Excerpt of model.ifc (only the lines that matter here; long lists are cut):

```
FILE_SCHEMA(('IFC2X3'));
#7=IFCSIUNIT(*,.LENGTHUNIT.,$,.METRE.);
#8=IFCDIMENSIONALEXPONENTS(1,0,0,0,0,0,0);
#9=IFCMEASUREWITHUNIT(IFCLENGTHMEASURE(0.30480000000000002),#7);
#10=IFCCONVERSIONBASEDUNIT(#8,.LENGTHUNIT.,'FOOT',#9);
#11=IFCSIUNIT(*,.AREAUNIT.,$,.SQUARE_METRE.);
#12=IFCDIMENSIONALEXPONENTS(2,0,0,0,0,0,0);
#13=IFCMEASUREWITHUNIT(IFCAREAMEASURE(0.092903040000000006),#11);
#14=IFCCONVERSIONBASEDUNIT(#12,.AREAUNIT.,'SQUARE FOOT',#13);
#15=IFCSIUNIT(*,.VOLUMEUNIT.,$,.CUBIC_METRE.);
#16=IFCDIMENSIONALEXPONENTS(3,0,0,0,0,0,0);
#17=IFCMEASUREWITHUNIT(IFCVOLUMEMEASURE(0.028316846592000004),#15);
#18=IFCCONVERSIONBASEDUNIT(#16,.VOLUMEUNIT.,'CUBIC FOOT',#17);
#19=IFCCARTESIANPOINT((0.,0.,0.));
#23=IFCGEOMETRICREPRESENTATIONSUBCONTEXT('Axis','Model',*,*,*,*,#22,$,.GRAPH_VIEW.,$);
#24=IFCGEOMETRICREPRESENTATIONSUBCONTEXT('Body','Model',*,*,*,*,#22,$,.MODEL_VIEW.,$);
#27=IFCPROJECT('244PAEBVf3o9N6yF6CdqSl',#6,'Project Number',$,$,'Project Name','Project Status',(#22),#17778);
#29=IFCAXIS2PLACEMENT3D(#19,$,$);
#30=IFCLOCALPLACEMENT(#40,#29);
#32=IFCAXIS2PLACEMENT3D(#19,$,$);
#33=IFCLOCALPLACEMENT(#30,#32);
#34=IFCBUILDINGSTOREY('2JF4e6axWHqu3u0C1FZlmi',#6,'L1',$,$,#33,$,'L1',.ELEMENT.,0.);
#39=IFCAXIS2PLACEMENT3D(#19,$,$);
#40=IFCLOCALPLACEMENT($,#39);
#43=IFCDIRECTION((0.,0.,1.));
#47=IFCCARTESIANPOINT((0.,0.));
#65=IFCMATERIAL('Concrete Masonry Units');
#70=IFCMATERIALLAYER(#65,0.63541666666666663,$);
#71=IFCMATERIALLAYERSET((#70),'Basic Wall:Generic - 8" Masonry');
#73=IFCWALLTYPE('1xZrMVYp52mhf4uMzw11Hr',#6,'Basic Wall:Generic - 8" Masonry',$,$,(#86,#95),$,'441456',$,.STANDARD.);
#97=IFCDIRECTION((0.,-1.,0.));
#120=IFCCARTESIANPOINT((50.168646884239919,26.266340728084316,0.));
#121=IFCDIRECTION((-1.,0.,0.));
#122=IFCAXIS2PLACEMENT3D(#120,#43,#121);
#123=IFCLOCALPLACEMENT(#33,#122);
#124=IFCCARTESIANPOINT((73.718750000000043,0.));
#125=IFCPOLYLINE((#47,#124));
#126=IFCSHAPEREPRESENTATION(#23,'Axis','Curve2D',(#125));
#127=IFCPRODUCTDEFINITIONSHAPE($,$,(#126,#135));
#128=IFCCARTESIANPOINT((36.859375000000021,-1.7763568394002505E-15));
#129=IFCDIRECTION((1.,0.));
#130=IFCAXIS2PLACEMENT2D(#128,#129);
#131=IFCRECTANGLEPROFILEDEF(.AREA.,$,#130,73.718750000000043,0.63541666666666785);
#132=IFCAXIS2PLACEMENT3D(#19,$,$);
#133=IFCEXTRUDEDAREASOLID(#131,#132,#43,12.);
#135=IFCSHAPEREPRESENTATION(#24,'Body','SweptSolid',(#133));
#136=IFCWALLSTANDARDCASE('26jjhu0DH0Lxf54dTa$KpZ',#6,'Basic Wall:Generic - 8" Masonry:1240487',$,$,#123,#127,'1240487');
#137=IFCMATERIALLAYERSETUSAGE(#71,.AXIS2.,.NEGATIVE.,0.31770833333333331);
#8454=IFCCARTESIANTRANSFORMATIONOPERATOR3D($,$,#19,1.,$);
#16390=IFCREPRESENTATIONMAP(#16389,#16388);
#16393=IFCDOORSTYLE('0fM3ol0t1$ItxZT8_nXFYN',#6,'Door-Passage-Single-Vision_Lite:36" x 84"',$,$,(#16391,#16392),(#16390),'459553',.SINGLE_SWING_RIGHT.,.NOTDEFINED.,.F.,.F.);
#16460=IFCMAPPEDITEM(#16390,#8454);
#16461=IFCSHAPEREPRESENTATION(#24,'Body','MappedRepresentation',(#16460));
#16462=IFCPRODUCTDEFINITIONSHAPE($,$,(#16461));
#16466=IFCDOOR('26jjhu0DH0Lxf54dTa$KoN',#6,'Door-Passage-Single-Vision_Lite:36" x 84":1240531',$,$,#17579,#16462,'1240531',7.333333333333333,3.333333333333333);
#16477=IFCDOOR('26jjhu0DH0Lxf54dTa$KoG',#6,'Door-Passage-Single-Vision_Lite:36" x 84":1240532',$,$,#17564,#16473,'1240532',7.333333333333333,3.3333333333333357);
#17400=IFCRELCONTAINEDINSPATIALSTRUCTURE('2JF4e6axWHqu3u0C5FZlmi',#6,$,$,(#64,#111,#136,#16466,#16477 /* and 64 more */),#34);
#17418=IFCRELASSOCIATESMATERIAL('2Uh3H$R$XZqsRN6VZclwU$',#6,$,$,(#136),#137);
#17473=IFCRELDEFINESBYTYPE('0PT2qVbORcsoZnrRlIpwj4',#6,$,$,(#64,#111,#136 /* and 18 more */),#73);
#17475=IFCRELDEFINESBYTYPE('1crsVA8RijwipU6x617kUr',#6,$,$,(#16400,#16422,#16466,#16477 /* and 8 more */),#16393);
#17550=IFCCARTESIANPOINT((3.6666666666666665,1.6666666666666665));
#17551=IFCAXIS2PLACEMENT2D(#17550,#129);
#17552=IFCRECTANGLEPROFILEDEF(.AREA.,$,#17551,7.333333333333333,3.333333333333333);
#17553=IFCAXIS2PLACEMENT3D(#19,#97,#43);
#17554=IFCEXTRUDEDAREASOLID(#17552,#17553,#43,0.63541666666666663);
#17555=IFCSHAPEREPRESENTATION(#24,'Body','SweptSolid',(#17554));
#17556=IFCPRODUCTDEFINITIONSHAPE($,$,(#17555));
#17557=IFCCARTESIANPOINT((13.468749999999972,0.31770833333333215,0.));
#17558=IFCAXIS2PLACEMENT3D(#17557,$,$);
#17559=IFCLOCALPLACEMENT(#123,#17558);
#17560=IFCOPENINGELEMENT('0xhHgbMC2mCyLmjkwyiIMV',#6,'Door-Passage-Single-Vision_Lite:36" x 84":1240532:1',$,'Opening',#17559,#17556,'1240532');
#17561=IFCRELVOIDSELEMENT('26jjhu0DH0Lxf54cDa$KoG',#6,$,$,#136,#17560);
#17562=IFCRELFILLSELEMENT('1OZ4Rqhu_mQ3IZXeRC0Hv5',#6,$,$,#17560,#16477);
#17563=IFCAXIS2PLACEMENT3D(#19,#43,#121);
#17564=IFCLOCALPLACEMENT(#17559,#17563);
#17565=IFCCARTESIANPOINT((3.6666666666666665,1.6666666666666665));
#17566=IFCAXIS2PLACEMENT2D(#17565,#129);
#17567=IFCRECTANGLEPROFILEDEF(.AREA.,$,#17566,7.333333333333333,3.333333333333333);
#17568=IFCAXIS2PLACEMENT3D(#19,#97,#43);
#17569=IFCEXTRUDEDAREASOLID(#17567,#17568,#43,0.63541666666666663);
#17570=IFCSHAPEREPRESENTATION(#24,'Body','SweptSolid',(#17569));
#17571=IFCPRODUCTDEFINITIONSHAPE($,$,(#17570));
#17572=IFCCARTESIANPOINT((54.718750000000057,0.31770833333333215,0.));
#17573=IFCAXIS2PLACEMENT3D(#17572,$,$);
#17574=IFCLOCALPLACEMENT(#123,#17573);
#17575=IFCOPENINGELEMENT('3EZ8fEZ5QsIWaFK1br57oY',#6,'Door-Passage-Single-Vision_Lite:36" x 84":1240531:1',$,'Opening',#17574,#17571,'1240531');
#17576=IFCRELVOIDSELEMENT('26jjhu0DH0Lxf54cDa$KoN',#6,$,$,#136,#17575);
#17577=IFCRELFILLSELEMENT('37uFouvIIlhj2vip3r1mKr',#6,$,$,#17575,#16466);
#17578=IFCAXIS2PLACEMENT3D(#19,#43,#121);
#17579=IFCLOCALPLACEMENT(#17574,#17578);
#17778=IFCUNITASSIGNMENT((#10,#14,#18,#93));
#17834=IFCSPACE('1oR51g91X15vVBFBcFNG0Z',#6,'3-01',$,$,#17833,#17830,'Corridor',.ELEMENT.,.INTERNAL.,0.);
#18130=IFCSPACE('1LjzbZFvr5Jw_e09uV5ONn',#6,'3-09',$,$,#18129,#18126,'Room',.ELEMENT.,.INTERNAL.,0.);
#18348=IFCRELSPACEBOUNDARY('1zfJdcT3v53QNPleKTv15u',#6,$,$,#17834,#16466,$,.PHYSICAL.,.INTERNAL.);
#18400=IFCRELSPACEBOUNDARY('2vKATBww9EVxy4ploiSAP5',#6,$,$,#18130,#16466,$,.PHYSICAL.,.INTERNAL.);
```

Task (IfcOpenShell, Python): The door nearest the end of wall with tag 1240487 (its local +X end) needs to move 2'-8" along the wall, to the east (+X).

```python
import ifcopenshell
import ifcopenshell.api.geometry
import ifcopenshell.util.placement
import ifcopenshell.util.unit

model = ifcopenshell.open("model.ifc")
unit_scale = ifcopenshell.util.unit.calculate_unit_scale(model)

door = model.by_guid("26jjhu0DH0Lxf54dTa$KoN")
opening = door.FillsVoids[0].RelatingOpeningElement
wall = opening.VoidsElements[0].RelatingBuildingElement

wall_matrix = ifcopenshell.util.placement.get_local_placement(wall.ObjectPlacement)
shift = wall_matrix[:3, 0] * -32 * 0.0254 / unit_scale
before = ifcopenshell.util.placement.get_local_placement(door.ObjectPlacement)[:3, 3].copy()

# The door is placed relative to its opening, so it follows when the opening moves.
matrix = ifcopenshell.util.placement.get_local_placement(opening.ObjectPlacement)
matrix[:3, 3] += shift
ifcopenshell.api.geometry.edit_object_placement(
    model, product=opening, matrix=matrix, is_si=False, should_transform_children=True
)

after = ifcopenshell.util.placement.get_local_placement(door.ObjectPlacement)[:3, 3]
print("door moved by", (after - before).round(3) + 0.0)

model.write("model-out.ifc")
```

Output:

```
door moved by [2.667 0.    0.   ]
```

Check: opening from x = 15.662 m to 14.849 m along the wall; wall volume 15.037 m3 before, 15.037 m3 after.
